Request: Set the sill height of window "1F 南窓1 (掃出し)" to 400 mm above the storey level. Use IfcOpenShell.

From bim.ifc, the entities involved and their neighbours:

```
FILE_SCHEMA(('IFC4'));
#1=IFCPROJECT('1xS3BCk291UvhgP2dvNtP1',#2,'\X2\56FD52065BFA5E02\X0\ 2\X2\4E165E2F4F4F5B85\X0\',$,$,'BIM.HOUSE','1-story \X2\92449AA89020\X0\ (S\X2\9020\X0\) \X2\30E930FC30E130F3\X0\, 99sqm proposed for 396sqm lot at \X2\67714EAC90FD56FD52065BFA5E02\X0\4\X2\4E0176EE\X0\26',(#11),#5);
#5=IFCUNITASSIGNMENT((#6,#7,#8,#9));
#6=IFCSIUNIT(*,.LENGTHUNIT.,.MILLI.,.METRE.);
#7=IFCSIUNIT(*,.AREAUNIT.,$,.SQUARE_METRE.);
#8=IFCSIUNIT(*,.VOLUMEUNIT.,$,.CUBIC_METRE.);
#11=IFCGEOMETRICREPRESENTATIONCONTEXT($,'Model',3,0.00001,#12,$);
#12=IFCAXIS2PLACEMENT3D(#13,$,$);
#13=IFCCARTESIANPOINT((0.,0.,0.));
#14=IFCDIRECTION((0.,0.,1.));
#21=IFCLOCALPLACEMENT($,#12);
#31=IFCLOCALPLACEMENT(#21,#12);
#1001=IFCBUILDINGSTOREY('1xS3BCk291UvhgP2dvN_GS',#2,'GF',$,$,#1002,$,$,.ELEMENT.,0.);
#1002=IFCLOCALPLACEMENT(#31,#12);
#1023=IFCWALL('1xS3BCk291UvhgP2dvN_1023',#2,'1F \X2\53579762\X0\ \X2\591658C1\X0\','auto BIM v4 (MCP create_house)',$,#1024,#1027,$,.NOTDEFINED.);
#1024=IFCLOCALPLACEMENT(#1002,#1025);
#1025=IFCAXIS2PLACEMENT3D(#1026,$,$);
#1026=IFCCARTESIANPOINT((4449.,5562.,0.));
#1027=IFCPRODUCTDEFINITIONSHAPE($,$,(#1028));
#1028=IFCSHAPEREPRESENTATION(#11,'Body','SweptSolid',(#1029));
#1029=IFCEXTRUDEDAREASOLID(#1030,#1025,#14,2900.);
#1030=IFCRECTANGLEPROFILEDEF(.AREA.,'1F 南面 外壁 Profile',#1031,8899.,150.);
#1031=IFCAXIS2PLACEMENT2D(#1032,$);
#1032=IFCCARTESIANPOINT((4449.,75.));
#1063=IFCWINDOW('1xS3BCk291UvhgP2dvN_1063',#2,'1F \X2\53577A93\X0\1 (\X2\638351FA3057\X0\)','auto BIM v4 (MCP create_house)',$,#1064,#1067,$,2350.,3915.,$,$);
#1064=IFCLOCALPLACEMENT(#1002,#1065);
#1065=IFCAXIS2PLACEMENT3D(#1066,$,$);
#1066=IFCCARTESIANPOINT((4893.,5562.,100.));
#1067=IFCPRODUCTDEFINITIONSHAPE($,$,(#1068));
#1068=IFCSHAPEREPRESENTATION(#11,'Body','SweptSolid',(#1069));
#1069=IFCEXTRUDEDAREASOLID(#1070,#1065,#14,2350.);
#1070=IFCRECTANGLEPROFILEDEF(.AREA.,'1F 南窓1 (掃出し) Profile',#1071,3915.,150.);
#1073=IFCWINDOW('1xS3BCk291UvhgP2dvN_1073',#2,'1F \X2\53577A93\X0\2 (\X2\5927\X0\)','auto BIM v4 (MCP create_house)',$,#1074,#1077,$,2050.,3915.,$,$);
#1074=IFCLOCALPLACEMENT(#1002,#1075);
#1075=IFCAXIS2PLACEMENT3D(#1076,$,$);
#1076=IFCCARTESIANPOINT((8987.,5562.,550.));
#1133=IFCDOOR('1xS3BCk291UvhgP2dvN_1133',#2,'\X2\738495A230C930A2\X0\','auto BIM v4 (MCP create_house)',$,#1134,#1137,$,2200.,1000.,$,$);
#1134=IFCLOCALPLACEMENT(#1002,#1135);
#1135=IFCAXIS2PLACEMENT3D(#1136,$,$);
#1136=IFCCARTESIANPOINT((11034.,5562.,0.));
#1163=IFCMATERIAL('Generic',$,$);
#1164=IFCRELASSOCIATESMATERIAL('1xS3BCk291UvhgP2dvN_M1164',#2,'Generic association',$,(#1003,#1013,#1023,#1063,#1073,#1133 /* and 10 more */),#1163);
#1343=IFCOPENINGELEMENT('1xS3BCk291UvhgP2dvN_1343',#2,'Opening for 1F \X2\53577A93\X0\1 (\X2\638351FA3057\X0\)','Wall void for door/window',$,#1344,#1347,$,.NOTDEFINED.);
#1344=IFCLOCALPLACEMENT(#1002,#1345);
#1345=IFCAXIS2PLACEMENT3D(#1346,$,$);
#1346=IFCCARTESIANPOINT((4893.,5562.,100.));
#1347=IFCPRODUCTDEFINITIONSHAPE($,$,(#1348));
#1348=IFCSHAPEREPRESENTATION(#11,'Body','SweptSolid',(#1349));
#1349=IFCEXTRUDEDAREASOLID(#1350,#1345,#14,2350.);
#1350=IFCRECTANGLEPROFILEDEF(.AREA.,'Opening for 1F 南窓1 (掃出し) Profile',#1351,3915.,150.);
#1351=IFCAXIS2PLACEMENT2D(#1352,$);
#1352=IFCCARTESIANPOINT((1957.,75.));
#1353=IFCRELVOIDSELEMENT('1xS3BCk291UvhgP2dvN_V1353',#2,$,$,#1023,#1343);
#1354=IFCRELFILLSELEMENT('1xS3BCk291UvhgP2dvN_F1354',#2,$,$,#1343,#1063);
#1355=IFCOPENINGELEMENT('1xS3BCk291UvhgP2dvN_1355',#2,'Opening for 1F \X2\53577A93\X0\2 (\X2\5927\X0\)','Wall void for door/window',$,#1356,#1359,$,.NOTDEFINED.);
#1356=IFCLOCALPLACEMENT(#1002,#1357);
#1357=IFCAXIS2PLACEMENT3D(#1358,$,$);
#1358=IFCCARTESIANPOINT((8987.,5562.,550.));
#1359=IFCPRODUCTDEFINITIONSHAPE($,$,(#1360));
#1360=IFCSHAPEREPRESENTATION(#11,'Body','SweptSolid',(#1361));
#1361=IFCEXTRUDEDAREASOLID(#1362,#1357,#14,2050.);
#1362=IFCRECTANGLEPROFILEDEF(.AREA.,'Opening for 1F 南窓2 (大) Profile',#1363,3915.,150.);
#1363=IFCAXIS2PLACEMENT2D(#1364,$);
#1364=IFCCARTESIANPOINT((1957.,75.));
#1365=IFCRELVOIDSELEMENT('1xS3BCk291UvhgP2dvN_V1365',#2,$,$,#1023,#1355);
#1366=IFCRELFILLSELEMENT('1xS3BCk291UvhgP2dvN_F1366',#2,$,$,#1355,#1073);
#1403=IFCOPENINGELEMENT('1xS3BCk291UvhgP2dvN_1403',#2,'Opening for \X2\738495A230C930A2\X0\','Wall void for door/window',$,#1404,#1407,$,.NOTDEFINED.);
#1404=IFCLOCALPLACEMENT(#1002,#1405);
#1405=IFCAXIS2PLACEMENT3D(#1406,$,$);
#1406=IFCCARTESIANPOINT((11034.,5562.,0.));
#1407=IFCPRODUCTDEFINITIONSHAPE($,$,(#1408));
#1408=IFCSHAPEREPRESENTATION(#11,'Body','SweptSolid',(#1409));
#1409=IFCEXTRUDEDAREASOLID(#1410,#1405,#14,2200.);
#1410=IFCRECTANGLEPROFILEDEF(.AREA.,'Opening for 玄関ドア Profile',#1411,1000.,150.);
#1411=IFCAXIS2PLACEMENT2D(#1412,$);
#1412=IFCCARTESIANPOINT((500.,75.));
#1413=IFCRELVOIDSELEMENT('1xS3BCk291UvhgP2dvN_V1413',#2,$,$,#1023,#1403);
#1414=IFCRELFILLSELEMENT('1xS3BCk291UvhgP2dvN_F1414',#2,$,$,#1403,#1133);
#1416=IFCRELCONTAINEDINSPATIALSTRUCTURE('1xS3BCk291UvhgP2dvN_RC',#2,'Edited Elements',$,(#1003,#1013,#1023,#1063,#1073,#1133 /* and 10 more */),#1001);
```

```python
import numpy as np
import ifcopenshell
import ifcopenshell.api.geometry
import ifcopenshell.geom
import ifcopenshell.util.element
import ifcopenshell.util.placement
import ifcopenshell.util.shape
import ifcopenshell.util.unit

model = ifcopenshell.open("bim.ifc")
unit_scale = ifcopenshell.util.unit.calculate_unit_scale(model)

window = model.by_guid("1xS3BCk291UvhgP2dvN_1063")
opening = window.FillsVoids[0].RelatingOpeningElement
storey = ifcopenshell.util.element.get_container(window, ifc_class="IfcBuildingStorey")
level = ifcopenshell.util.placement.get_local_placement(storey.ObjectPlacement)[2, 3]

# The opening's origin need not be at the sill, so measure its lowest point.
shape = ifcopenshell.geom.create_shape(ifcopenshell.geom.settings(), opening)
bottom = ifcopenshell.util.shape.get_shape_bottom_elevation(shape, shape.geometry) / unit_scale
dz = level + 400.0 - bottom

shift = np.array([0.0, 0.0, dz])
# The window is not placed relative to its opening, so move both.
for product in (opening, window):
    matrix = ifcopenshell.util.placement.get_local_placement(product.ObjectPlacement)
    matrix[:3, 3] += shift
    ifcopenshell.api.geometry.edit_object_placement(model, product=product, matrix=matrix, is_si=False)

print(f"moved by {dz * unit_scale:+.3f} m")

model.write("bim_rev.ifc")
```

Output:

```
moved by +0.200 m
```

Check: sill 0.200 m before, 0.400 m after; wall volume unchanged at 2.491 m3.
